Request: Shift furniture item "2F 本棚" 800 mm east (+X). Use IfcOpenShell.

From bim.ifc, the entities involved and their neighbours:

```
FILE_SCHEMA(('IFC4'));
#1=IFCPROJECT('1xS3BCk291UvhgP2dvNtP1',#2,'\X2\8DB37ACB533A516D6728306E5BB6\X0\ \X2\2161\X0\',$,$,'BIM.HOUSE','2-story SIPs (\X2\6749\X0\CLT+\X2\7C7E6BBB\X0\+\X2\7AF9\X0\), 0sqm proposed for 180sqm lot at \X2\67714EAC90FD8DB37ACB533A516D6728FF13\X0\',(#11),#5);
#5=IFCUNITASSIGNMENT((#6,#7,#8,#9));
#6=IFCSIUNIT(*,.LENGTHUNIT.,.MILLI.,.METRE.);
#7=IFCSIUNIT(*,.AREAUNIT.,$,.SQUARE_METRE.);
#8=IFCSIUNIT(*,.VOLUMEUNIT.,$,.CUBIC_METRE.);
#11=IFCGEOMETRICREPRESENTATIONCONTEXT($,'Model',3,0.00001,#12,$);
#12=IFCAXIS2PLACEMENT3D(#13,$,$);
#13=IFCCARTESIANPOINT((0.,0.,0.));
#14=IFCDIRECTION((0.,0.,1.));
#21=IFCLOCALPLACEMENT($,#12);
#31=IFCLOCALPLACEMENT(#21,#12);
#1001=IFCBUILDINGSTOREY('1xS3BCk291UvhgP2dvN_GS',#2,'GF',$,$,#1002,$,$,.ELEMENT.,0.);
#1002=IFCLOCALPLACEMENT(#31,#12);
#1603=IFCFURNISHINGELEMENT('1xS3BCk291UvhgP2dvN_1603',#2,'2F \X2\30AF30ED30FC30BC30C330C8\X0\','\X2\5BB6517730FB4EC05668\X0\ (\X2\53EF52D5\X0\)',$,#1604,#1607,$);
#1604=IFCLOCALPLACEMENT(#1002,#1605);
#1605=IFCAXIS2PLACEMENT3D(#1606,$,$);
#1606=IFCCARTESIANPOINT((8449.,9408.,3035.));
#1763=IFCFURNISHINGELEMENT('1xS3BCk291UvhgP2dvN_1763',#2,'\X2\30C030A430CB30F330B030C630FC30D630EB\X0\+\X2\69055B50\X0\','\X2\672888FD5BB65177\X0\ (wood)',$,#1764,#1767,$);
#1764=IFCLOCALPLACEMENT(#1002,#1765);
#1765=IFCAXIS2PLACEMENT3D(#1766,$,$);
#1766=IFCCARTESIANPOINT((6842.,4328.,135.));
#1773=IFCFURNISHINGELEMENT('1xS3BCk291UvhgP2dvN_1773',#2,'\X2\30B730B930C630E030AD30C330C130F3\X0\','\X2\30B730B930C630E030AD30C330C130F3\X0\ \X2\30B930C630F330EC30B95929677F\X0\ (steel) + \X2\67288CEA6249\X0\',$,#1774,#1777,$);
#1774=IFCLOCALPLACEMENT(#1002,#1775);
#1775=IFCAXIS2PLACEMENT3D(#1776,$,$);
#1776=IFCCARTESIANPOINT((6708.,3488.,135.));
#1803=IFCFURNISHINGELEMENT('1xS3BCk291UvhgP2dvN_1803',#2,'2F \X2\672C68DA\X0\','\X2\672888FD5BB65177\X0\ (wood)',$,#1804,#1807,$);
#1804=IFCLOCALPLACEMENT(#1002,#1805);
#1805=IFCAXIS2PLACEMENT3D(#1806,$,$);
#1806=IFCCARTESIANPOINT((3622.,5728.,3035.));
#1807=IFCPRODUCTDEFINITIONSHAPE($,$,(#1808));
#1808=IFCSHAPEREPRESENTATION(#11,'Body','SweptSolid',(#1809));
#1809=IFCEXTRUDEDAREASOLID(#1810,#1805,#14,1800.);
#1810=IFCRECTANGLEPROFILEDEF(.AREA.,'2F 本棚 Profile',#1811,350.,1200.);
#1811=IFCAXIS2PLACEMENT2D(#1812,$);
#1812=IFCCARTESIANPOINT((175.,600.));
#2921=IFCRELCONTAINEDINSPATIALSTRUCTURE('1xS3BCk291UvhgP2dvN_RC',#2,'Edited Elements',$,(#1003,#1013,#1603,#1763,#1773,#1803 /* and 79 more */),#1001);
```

```python
import ifcopenshell
import ifcopenshell.api.geometry
import ifcopenshell.util.placement
import ifcopenshell.util.unit

model = ifcopenshell.open("bim.ifc")
unit_scale = ifcopenshell.util.unit.calculate_unit_scale(model)

item = model.by_guid("1xS3BCk291UvhgP2dvN_1803")
matrix = ifcopenshell.util.placement.get_local_placement(item.ObjectPlacement)
matrix[0, 3] += 0.8 / unit_scale
ifcopenshell.api.geometry.edit_object_placement(model, product=item, matrix=matrix, is_si=False)

print(ifcopenshell.util.placement.get_local_placement(item.ObjectPlacement).round(3) + 0.0)

model.write("bim-out.ifc")
```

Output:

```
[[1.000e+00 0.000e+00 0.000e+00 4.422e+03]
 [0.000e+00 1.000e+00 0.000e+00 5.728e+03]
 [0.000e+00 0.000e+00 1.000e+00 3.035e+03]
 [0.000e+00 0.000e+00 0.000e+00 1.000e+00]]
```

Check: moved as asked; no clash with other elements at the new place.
